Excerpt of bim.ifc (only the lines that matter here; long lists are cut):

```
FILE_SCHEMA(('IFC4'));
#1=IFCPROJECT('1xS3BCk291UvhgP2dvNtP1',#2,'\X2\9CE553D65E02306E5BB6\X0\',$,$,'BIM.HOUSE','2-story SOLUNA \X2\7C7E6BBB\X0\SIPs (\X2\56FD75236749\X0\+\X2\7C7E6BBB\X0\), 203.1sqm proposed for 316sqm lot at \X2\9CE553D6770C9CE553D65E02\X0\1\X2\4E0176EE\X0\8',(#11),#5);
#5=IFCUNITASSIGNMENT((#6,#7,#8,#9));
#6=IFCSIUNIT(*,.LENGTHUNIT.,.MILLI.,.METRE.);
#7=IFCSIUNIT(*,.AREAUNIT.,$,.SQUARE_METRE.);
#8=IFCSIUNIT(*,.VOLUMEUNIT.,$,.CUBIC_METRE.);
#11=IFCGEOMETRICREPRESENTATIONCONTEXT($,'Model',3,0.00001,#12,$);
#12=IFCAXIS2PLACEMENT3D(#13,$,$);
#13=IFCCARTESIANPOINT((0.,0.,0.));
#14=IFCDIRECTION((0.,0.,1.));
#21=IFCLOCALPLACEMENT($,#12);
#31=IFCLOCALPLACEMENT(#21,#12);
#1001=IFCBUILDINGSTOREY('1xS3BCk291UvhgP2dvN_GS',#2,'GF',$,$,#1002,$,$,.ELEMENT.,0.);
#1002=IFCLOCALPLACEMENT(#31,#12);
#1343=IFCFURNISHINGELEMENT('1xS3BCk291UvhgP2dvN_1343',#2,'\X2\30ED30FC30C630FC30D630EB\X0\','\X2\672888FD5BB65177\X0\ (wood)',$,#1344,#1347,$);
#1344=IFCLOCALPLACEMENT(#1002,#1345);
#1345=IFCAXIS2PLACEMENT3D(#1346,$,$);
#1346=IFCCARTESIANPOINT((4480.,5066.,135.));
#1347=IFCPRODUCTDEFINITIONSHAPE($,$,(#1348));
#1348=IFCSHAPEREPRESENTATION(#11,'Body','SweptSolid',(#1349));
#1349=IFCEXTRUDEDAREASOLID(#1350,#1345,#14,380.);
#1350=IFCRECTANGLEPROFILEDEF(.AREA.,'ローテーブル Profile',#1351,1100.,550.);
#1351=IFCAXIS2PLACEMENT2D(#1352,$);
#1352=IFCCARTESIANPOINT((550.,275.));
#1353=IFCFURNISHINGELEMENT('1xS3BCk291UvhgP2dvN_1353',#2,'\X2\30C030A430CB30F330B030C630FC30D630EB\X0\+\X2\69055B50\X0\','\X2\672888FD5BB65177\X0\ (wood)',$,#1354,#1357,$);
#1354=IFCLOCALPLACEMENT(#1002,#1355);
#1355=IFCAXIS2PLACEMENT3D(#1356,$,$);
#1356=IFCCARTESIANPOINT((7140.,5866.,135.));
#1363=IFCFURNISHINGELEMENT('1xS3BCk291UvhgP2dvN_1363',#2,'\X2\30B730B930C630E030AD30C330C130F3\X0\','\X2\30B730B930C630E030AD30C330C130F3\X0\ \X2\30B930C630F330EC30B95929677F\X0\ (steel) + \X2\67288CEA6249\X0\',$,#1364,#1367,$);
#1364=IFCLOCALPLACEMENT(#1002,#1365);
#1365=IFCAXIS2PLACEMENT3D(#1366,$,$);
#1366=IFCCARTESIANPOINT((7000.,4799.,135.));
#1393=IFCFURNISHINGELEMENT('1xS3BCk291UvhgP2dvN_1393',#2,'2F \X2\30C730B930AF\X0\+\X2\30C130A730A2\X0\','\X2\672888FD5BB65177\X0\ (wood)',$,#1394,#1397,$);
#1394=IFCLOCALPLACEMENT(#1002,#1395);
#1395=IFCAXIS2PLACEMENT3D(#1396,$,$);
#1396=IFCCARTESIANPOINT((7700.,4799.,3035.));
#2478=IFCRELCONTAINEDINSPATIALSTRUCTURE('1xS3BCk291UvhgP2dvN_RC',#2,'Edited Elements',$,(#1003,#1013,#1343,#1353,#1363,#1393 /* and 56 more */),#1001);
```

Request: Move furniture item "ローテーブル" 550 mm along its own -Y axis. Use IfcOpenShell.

```python
import ifcopenshell
import ifcopenshell.api.geometry
import ifcopenshell.util.placement
import ifcopenshell.util.unit

model = ifcopenshell.open("bim.ifc")
unit_scale = ifcopenshell.util.unit.calculate_unit_scale(model)

item = model.by_guid("1xS3BCk291UvhgP2dvN_1343")
matrix = ifcopenshell.util.placement.get_local_placement(item.ObjectPlacement)
matrix[:3, 3] -= matrix[:3, 1] * 0.55 / unit_scale
ifcopenshell.api.geometry.edit_object_placement(model, product=item, matrix=matrix, is_si=False)

print(ifcopenshell.util.placement.get_local_placement(item.ObjectPlacement).round(3) + 0.0)

model.write("bim_edited.ifc")
```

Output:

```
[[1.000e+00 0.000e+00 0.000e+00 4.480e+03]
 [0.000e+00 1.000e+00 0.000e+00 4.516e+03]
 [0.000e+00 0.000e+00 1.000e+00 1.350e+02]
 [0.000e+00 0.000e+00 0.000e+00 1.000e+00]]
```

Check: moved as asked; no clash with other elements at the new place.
